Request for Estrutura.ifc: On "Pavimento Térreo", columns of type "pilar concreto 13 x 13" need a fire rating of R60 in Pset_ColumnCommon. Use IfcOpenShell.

First a look at what the model holds.

```python
import ifcopenshell
import ifcopenshell.util.element

model = ifcopenshell.open("Estrutura.ifc")
print(model.schema)
storey = next(s for s in model.by_type("IfcBuildingStorey") if s.Name == "Pavimento Térreo")
columns = [e for e in ifcopenshell.util.element.get_decomposition(storey) if e.is_a("IfcColumn")]
seen = {}
for e in columns:
    element_type = ifcopenshell.util.element.get_type(e)
    key = (element_type.Name if element_type != e and element_type else None, ifcopenshell.util.element.get_pset(e, "Pset_ColumnCommon", "FireRating"))
    seen[key] = seen.get(key, 0) + 1
for (name, value), count in sorted(seen.items(), key=str):
    print(count, "x", name, "|", value)
```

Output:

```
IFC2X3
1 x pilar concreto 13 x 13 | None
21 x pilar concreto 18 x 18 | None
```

```python
import ifcopenshell
import ifcopenshell.api.pset
import ifcopenshell.util.element

model = ifcopenshell.open("Estrutura.ifc")

storey = next(s for s in model.by_type("IfcBuildingStorey") if s.Name == "Pavimento Térreo")
columns = [e for e in ifcopenshell.util.element.get_decomposition(storey) if e.is_a("IfcColumn")]

count = 0
for e in columns:
    element_type = ifcopenshell.util.element.get_type(e)
    if element_type in (None, e) or element_type.Name != "pilar concreto 13 x 13":
        continue
    # add_pset returns the element's existing set when there is one.
    pset = ifcopenshell.api.pset.add_pset(model, product=e, name="Pset_ColumnCommon")
    ifcopenshell.api.pset.edit_pset(model, pset=pset, properties={"FireRating": "R60"})
    count += 1

print(count, "columns updated")

model.write("Estrutura_v2.ifc")
```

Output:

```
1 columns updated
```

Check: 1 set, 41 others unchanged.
